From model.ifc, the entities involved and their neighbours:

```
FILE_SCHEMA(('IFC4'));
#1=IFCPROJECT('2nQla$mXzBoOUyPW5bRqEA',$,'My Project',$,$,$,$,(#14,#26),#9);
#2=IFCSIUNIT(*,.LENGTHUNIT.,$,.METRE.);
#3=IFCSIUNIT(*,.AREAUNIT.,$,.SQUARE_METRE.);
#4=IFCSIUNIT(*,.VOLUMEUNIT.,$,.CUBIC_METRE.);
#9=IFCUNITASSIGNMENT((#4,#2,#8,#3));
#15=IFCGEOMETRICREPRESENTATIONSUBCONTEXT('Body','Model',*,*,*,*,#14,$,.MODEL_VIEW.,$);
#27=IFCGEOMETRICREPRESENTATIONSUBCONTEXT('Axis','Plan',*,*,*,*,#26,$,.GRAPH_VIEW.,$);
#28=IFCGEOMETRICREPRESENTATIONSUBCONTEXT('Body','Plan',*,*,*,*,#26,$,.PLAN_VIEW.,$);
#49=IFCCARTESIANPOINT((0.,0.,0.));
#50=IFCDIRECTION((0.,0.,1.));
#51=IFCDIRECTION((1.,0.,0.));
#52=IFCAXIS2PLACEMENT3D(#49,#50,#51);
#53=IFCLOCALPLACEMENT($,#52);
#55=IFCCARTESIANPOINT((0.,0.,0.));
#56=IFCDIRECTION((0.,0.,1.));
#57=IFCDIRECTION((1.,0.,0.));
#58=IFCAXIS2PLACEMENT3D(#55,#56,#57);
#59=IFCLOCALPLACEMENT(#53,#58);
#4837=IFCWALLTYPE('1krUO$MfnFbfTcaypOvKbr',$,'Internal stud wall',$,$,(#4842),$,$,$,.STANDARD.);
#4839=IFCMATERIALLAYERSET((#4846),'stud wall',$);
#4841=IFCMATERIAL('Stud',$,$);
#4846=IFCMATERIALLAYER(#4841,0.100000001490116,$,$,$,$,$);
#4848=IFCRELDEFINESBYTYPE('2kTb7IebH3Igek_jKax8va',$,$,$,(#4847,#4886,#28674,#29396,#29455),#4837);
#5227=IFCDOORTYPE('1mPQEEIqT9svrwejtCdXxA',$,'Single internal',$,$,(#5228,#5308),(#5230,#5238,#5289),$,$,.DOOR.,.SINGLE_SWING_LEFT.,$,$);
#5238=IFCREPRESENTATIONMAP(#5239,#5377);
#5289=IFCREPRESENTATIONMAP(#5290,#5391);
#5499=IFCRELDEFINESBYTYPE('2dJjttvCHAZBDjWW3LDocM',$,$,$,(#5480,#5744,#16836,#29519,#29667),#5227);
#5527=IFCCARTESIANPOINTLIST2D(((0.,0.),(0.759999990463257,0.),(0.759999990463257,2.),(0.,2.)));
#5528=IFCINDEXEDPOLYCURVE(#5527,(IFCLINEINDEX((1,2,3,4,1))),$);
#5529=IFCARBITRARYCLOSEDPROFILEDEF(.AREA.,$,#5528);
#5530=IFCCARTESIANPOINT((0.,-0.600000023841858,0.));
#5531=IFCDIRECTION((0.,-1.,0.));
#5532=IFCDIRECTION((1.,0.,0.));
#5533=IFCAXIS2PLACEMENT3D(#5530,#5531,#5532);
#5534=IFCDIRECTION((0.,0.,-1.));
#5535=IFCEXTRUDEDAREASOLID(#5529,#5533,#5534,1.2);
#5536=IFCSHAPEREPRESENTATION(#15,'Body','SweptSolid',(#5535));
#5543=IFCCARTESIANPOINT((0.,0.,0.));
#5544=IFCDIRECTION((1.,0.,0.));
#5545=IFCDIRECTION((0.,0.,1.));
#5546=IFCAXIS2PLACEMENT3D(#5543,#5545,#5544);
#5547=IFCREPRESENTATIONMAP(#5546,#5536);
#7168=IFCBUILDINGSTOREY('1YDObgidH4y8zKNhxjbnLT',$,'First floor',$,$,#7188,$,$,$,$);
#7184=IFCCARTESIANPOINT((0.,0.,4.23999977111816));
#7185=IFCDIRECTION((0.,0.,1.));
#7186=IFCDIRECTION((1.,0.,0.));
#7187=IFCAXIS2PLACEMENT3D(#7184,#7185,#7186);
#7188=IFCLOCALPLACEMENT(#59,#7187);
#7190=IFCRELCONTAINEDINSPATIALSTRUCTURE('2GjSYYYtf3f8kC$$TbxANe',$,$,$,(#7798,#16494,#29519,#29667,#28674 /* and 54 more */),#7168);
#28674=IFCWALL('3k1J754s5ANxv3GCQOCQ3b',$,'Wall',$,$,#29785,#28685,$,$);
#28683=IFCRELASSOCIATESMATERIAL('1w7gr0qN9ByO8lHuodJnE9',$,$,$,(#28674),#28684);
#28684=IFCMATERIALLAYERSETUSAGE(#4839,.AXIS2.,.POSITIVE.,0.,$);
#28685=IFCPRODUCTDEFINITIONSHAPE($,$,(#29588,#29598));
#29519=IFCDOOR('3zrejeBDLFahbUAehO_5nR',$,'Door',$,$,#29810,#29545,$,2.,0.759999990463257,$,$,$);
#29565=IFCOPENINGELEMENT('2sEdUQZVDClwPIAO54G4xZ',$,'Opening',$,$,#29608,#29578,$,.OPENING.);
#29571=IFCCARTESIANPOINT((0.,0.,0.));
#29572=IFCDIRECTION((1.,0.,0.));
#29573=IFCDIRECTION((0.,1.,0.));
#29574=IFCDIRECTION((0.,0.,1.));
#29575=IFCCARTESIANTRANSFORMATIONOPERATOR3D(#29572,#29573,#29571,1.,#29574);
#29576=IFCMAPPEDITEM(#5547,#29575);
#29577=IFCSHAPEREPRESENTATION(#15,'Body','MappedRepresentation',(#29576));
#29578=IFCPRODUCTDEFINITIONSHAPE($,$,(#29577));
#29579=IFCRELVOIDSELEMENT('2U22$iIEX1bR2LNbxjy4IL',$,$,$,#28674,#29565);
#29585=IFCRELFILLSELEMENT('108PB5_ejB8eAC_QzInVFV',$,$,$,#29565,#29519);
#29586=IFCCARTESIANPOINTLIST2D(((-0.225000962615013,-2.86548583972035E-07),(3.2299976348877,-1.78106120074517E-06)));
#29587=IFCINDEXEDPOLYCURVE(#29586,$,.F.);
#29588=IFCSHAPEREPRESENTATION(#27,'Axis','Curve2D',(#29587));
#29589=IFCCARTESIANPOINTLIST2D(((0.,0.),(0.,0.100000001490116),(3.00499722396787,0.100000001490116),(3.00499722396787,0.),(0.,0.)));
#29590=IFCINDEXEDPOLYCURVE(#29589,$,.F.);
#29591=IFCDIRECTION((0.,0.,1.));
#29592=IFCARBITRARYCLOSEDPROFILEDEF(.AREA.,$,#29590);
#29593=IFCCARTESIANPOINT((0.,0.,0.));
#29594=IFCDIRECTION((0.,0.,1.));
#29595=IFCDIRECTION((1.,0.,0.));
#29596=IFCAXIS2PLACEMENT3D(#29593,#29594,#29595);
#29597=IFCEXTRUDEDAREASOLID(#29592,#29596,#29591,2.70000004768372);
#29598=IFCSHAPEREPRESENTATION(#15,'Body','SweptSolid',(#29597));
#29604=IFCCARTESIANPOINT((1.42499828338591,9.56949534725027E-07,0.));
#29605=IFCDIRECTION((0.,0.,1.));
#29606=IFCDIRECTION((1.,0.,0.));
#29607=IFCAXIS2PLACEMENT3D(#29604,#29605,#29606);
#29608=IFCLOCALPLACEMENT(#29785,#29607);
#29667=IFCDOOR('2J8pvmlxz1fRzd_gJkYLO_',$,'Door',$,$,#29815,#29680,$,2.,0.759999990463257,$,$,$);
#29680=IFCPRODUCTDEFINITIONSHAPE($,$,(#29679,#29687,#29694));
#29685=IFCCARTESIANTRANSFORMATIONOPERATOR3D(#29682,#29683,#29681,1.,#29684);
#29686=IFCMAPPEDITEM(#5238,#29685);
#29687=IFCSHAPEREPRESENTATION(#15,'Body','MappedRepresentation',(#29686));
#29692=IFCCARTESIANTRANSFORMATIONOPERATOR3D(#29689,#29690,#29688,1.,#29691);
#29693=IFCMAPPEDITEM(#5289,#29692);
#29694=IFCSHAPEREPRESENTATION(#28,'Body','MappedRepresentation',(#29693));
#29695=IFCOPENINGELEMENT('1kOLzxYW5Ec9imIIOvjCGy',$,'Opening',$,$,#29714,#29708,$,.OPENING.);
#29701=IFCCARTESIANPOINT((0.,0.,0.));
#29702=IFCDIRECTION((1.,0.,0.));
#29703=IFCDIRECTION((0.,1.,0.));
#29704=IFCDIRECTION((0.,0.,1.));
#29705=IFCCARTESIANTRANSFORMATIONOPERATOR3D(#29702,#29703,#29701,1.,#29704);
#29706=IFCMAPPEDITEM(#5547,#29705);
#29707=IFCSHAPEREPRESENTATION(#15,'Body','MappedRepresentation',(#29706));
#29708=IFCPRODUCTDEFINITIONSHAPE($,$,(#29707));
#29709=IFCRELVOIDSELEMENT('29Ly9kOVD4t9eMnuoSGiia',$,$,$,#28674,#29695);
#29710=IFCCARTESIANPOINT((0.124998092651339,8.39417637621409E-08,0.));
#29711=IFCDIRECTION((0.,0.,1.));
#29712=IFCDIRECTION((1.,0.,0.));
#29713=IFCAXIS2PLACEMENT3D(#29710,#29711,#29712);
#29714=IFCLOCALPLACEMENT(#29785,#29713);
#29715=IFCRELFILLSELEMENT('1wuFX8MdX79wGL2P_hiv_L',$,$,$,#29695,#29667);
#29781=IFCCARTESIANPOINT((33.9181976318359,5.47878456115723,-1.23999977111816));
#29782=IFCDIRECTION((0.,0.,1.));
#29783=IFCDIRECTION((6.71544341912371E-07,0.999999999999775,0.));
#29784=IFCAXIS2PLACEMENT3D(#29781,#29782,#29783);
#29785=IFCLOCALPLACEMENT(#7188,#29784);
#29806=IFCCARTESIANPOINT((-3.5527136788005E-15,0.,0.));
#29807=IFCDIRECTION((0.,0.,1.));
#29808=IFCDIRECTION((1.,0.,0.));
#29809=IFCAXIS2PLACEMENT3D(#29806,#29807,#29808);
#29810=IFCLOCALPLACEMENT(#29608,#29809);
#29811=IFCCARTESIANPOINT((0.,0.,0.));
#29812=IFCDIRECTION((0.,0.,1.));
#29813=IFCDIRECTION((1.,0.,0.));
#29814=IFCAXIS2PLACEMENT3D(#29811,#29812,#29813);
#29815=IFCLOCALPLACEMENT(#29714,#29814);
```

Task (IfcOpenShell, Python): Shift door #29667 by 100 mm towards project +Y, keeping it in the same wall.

```python
import ifcopenshell
import ifcopenshell.api.geometry
import ifcopenshell.util.placement

model = ifcopenshell.open("model.ifc")

door = model.by_guid("2J8pvmlxz1fRzd_gJkYLO_")
opening = door.FillsVoids[0].RelatingOpeningElement
wall = opening.VoidsElements[0].RelatingBuildingElement

wall_matrix = ifcopenshell.util.placement.get_local_placement(wall.ObjectPlacement)
shift = wall_matrix[:3, 0] * 0.1
before = ifcopenshell.util.placement.get_local_placement(door.ObjectPlacement)[:3, 3].copy()

# The door is placed relative to its opening, so it follows when the opening moves.
matrix = ifcopenshell.util.placement.get_local_placement(opening.ObjectPlacement)
matrix[:3, 3] += shift
ifcopenshell.api.geometry.edit_object_placement(
    model, product=opening, matrix=matrix, is_si=False, should_transform_children=True
)

after = ifcopenshell.util.placement.get_local_placement(door.ObjectPlacement)[:3, 3]
print("door moved by", (after - before).round(3) + 0.0)

model.write("model_updated.ifc")
```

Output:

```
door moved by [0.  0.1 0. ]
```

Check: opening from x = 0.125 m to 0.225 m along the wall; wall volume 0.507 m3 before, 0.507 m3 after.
